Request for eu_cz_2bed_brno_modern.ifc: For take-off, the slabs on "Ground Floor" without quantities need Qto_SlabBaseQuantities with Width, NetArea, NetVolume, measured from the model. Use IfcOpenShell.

First a look at what the model holds.

```python
import ifcopenshell
import ifcopenshell.util.element
import ifcopenshell.util.unit

model = ifcopenshell.open("eu_cz_2bed_brno_modern.ifc")
print(model.schema)
for unit_type in ("LENGTHUNIT", "AREAUNIT", "VOLUMEUNIT"):
    print(unit_type, ifcopenshell.util.unit.calculate_unit_scale(model, unit_type))
storey = next(s for s in model.by_type("IfcBuildingStorey") if s.Name == "Ground Floor")
slabs = [e for e in ifcopenshell.util.element.get_decomposition(storey) if e.is_a("IfcSlab")]
for e in sorted(slabs, key=lambda e: e.id()):
    print(e.id(), e.is_a(), e.Name, list(ifcopenshell.util.element.get_psets(e, qtos_only=True)), sep=" | ")
```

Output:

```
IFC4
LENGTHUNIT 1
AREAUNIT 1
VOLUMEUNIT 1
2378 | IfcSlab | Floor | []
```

```python
import ifcopenshell
import ifcopenshell.api.pset
import ifcopenshell.geom
import ifcopenshell.util.element
import ifcopenshell.util.shape
import ifcopenshell.util.unit

model = ifcopenshell.open("eu_cz_2bed_brno_modern.ifc")
unit_scale = ifcopenshell.util.unit.calculate_unit_scale(model)
area_scale = ifcopenshell.util.unit.calculate_unit_scale(model, "AREAUNIT")
volume_scale = ifcopenshell.util.unit.calculate_unit_scale(model, "VOLUMEUNIT")
settings = ifcopenshell.geom.settings()

storey = next(s for s in model.by_type("IfcBuildingStorey") if s.Name == "Ground Floor")
slabs = [e for e in ifcopenshell.util.element.get_decomposition(storey) if e.is_a("IfcSlab")]

for e in sorted(slabs, key=lambda e: e.id()):
    if ifcopenshell.util.element.get_psets(e, qtos_only=True, should_inherit=False):
        continue
    # Geometry comes back in metres, in the element's own axes.
    shape = ifcopenshell.geom.create_shape(settings, e)
    values = {
        "Width": ifcopenshell.util.shape.get_z(shape.geometry) / unit_scale,
        "NetArea": ifcopenshell.util.shape.get_footprint_area(shape.geometry) / area_scale,
        "NetVolume": ifcopenshell.util.shape.get_volume(shape.geometry) / volume_scale,
    }
    qto = ifcopenshell.api.pset.add_qto(model, product=e, name="Qto_SlabBaseQuantities")
    ifcopenshell.api.pset.edit_qto(model, qto=qto, properties=values)
    print(e.id(), {k: round(v, 3) for k, v in values.items()})

model.write("eu_cz_2bed_brno_modern-out.ifc")
```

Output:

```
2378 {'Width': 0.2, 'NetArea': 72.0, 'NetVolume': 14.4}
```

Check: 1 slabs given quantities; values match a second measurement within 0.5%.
